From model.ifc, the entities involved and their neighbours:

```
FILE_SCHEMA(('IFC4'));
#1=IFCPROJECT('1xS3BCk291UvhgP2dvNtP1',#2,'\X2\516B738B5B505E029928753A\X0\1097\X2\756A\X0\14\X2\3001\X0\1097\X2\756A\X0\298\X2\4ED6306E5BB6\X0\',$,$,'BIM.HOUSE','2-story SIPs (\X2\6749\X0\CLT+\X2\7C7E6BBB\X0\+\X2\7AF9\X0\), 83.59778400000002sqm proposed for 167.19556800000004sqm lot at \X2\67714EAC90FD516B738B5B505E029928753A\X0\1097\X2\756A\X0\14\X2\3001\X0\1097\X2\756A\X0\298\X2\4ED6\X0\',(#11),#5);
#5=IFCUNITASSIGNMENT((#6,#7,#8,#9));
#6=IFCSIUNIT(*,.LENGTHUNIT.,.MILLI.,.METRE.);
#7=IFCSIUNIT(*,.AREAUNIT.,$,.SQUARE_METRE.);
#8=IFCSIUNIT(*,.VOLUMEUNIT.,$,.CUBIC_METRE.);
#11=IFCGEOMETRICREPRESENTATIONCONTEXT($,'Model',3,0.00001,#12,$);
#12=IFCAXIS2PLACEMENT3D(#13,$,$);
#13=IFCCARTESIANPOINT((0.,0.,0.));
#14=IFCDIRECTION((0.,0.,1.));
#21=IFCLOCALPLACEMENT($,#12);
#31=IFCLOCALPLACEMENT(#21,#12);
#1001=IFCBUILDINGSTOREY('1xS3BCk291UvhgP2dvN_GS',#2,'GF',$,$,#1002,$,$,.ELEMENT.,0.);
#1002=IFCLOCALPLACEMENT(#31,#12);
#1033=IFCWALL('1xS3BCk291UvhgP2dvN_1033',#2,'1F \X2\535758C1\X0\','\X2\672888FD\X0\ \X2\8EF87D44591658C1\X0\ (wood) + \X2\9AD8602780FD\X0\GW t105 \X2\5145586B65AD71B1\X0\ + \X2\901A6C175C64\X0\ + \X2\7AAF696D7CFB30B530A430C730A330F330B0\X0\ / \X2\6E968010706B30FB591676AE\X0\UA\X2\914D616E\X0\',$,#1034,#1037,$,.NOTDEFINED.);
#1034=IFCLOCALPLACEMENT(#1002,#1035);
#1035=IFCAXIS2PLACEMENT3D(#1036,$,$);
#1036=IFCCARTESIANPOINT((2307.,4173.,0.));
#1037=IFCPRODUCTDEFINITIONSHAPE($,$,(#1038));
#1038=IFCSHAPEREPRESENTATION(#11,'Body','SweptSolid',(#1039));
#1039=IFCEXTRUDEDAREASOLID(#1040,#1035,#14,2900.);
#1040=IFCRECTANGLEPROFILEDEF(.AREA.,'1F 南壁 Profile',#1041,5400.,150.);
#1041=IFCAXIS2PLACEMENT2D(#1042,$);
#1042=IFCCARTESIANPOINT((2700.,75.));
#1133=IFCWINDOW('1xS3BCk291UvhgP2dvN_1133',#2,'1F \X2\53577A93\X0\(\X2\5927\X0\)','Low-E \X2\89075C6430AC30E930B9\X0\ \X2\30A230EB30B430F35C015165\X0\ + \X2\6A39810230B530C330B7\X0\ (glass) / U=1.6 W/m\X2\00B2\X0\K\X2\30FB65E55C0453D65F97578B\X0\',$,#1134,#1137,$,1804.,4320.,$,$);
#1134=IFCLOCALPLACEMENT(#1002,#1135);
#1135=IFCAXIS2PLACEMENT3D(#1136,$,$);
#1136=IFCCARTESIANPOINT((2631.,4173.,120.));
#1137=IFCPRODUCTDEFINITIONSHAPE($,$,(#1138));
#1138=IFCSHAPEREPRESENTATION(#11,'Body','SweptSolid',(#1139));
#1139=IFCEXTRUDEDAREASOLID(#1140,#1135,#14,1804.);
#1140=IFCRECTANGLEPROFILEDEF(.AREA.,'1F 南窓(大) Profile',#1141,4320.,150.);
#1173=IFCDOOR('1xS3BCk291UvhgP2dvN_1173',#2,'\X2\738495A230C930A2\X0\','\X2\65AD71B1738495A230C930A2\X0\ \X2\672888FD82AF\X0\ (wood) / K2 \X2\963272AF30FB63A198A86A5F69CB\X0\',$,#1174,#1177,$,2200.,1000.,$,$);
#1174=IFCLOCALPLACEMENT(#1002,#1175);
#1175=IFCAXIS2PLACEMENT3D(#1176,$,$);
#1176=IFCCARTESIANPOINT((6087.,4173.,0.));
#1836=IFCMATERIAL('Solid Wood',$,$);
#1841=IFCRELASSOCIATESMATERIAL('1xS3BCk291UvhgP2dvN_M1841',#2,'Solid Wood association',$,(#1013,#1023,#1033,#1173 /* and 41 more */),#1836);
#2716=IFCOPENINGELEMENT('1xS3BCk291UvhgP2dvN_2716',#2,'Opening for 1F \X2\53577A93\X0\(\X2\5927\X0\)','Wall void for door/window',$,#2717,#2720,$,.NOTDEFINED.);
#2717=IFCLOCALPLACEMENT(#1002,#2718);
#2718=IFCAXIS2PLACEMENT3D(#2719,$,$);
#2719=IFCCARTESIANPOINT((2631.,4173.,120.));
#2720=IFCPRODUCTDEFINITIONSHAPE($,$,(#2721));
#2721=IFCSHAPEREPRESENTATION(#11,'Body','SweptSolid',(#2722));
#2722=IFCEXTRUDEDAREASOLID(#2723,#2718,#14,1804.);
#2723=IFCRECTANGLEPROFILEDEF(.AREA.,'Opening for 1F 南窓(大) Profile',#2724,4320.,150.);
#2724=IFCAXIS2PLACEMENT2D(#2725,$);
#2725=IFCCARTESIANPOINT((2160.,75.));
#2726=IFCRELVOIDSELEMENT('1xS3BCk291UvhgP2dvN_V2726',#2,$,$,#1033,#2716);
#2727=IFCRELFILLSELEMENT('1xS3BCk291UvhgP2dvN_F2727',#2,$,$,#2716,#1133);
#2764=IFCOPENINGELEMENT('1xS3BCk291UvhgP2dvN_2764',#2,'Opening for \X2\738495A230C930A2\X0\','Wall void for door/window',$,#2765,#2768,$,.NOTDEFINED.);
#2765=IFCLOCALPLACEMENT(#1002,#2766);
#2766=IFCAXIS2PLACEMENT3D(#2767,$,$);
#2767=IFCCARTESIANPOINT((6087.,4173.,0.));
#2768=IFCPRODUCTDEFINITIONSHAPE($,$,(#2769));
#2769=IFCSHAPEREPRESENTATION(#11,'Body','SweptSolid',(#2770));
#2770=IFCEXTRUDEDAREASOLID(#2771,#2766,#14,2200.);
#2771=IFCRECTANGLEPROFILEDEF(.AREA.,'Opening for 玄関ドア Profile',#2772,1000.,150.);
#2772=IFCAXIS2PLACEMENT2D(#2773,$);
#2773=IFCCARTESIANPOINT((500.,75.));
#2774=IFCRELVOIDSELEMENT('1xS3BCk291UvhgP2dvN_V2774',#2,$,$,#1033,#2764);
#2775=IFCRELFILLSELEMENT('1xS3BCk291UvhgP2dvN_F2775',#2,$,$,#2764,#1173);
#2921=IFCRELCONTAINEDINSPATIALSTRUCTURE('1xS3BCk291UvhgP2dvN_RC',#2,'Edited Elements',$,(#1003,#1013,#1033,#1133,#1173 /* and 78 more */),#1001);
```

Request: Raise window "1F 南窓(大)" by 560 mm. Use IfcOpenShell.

```python
import numpy as np
import ifcopenshell
import ifcopenshell.api.geometry
import ifcopenshell.util.placement
import ifcopenshell.util.unit

model = ifcopenshell.open("model.ifc")
unit_scale = ifcopenshell.util.unit.calculate_unit_scale(model)

window = model.by_guid("1xS3BCk291UvhgP2dvN_1133")
opening = window.FillsVoids[0].RelatingOpeningElement
dz = 560.0

shift = np.array([0.0, 0.0, dz])
# The window is not placed relative to its opening, so move both.
for product in (opening, window):
    matrix = ifcopenshell.util.placement.get_local_placement(product.ObjectPlacement)
    matrix[:3, 3] += shift
    ifcopenshell.api.geometry.edit_object_placement(model, product=product, matrix=matrix, is_si=False)

print(f"moved by {dz * unit_scale:+.3f} m")

model.write("model-out.ifc")
```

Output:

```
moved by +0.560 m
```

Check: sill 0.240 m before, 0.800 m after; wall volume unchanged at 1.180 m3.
